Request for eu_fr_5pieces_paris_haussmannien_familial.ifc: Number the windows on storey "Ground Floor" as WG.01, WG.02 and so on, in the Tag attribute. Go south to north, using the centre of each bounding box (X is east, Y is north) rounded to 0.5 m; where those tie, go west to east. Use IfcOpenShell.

First a look at what the model holds.

```python
import ifcopenshell
import ifcopenshell.util.element
import ifcopenshell.util.placement

model = ifcopenshell.open("eu_fr_5pieces_paris_haussmannien_familial.ifc")
print(model.schema)
storey = next(s for s in model.by_type("IfcBuildingStorey") if s.Name == "Ground Floor")
windows = [e for e in ifcopenshell.util.element.get_decomposition(storey) if e.is_a("IfcWindow")]
for e in sorted(windows, key=lambda e: e.id()):
    origin = ifcopenshell.util.placement.get_local_placement(e.ObjectPlacement)[:3, 3]
    print(e.id(), e.Tag, e.Name, origin.round(2) + 0.0, sep=" | ")
```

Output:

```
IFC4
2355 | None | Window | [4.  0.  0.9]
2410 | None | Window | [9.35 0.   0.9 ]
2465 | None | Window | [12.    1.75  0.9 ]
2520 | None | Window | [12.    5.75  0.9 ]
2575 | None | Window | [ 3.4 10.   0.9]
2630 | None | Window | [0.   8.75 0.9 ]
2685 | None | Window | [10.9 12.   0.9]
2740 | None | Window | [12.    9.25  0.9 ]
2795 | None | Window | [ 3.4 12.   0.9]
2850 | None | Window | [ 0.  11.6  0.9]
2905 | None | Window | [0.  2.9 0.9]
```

```python
import ifcopenshell
import ifcopenshell.geom
import ifcopenshell.util.element
import ifcopenshell.util.shape

model = ifcopenshell.open("eu_fr_5pieces_paris_haussmannien_familial.ifc")
settings = ifcopenshell.geom.settings()
settings.set("use-world-coords", True)


def centre(element):
    shape = ifcopenshell.geom.create_shape(settings, element)
    return ifcopenshell.util.shape.get_bbox_centroid(shape.geometry)


storey = next(s for s in model.by_type("IfcBuildingStorey") if s.Name == "Ground Floor")
windows = [e for e in ifcopenshell.util.element.get_decomposition(storey) if e.is_a("IfcWindow")]

# Insertion points can sit at a corner or the storey origin, so sort by the geometry (in metres).
centres = {e: centre(e) for e in windows}
windows.sort(key=lambda e: (round(centres[e][1] / 0.5), centres[e][0]))

for i, e in enumerate(windows, start=1):
    number = f"WG.{i:02d}"
    e.Tag = number
    print(e.id(), number)

model.write("eu_fr_5pieces_paris_haussmannien_familial_v2.ifc")
```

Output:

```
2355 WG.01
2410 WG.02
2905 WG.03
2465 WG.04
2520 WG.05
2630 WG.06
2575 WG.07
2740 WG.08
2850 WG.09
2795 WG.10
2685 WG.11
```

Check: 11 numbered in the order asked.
